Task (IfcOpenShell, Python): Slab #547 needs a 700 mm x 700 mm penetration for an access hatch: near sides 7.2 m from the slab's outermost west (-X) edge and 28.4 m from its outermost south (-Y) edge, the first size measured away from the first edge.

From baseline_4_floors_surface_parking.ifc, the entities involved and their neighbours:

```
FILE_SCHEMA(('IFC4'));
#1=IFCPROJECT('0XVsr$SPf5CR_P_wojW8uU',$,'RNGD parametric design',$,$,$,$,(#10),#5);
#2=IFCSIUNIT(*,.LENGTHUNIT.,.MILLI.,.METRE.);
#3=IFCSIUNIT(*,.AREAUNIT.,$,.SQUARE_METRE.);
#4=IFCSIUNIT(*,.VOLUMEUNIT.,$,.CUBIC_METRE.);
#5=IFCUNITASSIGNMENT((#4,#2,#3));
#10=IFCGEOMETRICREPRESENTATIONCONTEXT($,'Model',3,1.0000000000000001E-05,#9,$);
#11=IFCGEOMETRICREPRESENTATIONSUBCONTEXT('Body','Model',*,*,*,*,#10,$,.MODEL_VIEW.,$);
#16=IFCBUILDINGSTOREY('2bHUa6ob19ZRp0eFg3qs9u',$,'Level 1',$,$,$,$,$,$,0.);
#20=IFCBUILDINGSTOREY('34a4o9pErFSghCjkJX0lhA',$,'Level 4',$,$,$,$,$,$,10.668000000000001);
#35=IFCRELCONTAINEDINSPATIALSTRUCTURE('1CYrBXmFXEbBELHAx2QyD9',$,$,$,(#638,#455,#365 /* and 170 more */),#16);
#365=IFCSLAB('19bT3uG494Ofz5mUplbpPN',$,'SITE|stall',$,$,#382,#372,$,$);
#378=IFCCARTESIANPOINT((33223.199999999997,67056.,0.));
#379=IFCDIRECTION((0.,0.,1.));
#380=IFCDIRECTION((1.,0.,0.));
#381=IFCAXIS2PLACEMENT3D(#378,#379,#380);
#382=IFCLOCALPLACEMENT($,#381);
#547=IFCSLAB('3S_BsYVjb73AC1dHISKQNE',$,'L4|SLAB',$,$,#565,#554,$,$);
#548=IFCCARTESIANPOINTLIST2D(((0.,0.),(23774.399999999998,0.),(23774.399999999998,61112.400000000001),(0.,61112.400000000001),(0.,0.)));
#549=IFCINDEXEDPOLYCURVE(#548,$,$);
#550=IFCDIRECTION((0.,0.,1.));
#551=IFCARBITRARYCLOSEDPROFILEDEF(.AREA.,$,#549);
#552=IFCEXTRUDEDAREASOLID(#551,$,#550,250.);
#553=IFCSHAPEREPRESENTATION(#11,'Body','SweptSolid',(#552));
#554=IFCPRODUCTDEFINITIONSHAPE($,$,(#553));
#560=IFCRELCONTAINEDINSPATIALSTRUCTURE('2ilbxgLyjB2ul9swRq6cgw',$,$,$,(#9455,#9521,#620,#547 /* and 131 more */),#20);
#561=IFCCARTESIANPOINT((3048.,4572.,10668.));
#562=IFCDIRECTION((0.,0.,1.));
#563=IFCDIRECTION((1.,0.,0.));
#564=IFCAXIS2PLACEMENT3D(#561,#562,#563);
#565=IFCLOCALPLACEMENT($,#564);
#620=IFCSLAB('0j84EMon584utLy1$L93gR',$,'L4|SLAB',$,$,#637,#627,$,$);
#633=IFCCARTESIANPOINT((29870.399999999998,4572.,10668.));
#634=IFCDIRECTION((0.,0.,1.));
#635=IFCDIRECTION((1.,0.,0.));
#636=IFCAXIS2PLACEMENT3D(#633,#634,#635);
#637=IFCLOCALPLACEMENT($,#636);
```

```python
import numpy as np
import ifcopenshell
import ifcopenshell.api.feature
import ifcopenshell.api.geometry
import ifcopenshell.api.root
import ifcopenshell.geom
import ifcopenshell.util.placement
import ifcopenshell.util.representation
import ifcopenshell.util.shape
import ifcopenshell.util.unit

model = ifcopenshell.open("baseline_4_floors_surface_parking.ifc")
unit_scale = ifcopenshell.util.unit.calculate_unit_scale(model)
settings = ifcopenshell.geom.settings()


def volume(element):
    """Net volume in cubic metres, openings subtracted."""
    shape = ifcopenshell.geom.create_shape(settings, element)
    return ifcopenshell.util.shape.get_volume(shape.geometry)


slab = model.by_guid("3S_BsYVjb73AC1dHISKQNE")
before = volume(slab)

# Extent in the slab's own axes, in metres. The edges named are its -X and -Y sides.
slab_shape = ifcopenshell.geom.create_shape(settings, slab)
vertices = ifcopenshell.util.shape.get_vertices(slab_shape.geometry)
x_min, y_min, bottom = vertices.min(axis=0)
top = vertices[:, 2].max()

opening = ifcopenshell.api.root.create_entity(model, ifc_class="IfcOpeningElement", name="Access hatch opening", predefined_type="OPENING")
context = ifcopenshell.util.representation.get_context(model, "Model", "Body", "MODEL_VIEW")
width, depth = 0.7, 0.7
outline = [(0.0, 0.0), (width, 0.0), (width, depth), (0.0, depth), (0.0, 0.0)]
# Overshoot both faces by 50 mm so the cut is clean.
shape = ifcopenshell.api.geometry.add_slab_representation(
    model, context=context, depth=top - bottom + 0.1, polyline=outline
)
ifcopenshell.api.geometry.assign_representation(model, product=opening, representation=shape)

matrix = ifcopenshell.util.placement.get_local_placement(slab.ObjectPlacement)
matrix[:, 3] = matrix @ np.append(np.array([x_min + 7.2, y_min + 28.4, bottom - 0.05]) / unit_scale, 1.0)
ifcopenshell.api.geometry.edit_object_placement(model, product=opening, matrix=matrix, is_si=False)
ifcopenshell.api.feature.add_feature(model, feature=opening, element=slab)

after = volume(slab)

print(f"slab volume {before:.3f} -> {after:.3f} m3")

model.write("baseline_4_floors_surface_parking_v2.ifc")
```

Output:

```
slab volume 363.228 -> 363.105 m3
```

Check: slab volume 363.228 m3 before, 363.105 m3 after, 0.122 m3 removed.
